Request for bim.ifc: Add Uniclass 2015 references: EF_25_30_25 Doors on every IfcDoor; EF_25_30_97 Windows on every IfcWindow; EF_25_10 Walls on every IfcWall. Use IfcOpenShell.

First a look at what the model holds.

```python
import ifcopenshell

model = ifcopenshell.open("bim.ifc")
print(model.schema)
print("classifications:", [c.Name for c in model.by_type("IfcClassification")])
for ifc_class in ("IfcDoor", "IfcRoof", "IfcStair", "IfcWall", "IfcWindow"):
    print(ifc_class, len(model.by_type(ifc_class)))
```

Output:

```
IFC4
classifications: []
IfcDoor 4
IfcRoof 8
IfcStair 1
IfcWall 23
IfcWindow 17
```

```python
import ifcopenshell
import ifcopenshell.api.classification

model = ifcopenshell.open("bim.ifc")

system = ifcopenshell.api.classification.add_classification(model, classification="Uniclass 2015")

codes = {
    "IfcDoor": ("EF_25_30_25", "Doors"),
    "IfcWindow": ("EF_25_30_97", "Windows"),
    "IfcWall": ("EF_25_10", "Walls"),
}
for ifc_class, (code, name) in codes.items():
    products = model.by_type(ifc_class)
    ifcopenshell.api.classification.add_reference(
        model, products=products, classification=system, identification=code, name=name
    )
    print(code, len(products))

model.write("bim_updated.ifc")
```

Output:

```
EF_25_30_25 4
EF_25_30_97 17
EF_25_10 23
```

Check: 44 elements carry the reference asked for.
